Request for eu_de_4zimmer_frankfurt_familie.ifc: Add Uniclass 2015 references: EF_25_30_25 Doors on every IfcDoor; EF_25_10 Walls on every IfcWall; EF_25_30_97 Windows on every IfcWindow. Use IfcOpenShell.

First a look at what the model holds.

```python
import ifcopenshell

model = ifcopenshell.open("eu_de_4zimmer_frankfurt_familie.ifc")
print(model.schema)
print("classifications:", [c.Name for c in model.by_type("IfcClassification")])
for ifc_class in ("IfcDoor", "IfcRoof", "IfcStair", "IfcWall", "IfcWindow"):
    print(ifc_class, len(model.by_type(ifc_class)))
```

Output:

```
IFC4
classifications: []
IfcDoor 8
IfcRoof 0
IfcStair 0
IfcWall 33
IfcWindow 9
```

```python
import ifcopenshell
import ifcopenshell.api.classification

model = ifcopenshell.open("eu_de_4zimmer_frankfurt_familie.ifc")

system = ifcopenshell.api.classification.add_classification(model, classification="Uniclass 2015")

codes = {
    "IfcDoor": ("EF_25_30_25", "Doors"),
    "IfcWall": ("EF_25_10", "Walls"),
    "IfcWindow": ("EF_25_30_97", "Windows"),
}
for ifc_class, (code, name) in codes.items():
    products = model.by_type(ifc_class)
    ifcopenshell.api.classification.add_reference(
        model, products=products, classification=system, identification=code, name=name
    )
    print(code, len(products))

model.write("eu_de_4zimmer_frankfurt_familie-out.ifc")
```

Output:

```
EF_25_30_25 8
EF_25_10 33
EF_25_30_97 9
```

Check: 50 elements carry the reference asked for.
